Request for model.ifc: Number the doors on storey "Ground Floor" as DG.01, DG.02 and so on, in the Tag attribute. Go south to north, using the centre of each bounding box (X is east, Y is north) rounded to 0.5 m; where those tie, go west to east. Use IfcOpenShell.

First a look at what the model holds.

```python
import ifcopenshell
import ifcopenshell.util.element
import ifcopenshell.util.placement

model = ifcopenshell.open("model.ifc")
print(model.schema)
storey = next(s for s in model.by_type("IfcBuildingStorey") if s.Name == "Ground Floor")
doors = [e for e in ifcopenshell.util.element.get_decomposition(storey) if e.is_a("IfcDoor")]
for e in sorted(doors, key=lambda e: e.id()):
    origin = ifcopenshell.util.placement.get_local_placement(e.ObjectPlacement)[:3, 3]
    print(e.id(), e.Tag, e.Name, origin.round(2) + 0.0, sep=" | ")
```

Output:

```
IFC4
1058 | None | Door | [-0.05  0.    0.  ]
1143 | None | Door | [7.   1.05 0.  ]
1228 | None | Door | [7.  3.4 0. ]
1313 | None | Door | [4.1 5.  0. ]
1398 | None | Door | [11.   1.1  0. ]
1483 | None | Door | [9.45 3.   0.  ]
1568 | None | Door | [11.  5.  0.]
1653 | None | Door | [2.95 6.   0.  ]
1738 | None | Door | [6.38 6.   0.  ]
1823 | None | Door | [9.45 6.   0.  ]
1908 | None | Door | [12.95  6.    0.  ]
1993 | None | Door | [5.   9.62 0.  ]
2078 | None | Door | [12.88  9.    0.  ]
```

```python
import ifcopenshell
import ifcopenshell.geom
import ifcopenshell.util.element
import ifcopenshell.util.shape

model = ifcopenshell.open("model.ifc")
settings = ifcopenshell.geom.settings()
settings.set("use-world-coords", True)


def centre(element):
    shape = ifcopenshell.geom.create_shape(settings, element)
    return ifcopenshell.util.shape.get_bbox_centroid(shape.geometry)


storey = next(s for s in model.by_type("IfcBuildingStorey") if s.Name == "Ground Floor")
doors = [e for e in ifcopenshell.util.element.get_decomposition(storey) if e.is_a("IfcDoor")]

# Insertion points can sit at a corner or the storey origin, so sort by the geometry (in metres).
centres = {e: centre(e) for e in doors}
doors.sort(key=lambda e: (round(centres[e][1] / 0.5), centres[e][0]))

for i, e in enumerate(doors, start=1):
    number = f"DG.{i:02d}"
    e.Tag = number
    print(e.id(), number)

model.write("model_rev.ifc")
```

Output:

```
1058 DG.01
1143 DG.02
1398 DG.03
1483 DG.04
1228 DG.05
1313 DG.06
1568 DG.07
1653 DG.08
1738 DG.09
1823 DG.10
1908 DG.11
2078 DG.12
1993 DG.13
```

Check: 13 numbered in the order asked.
